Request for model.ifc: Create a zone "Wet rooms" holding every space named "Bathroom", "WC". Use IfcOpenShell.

First a look at what the model holds.

```python
import ifcopenshell

model = ifcopenshell.open("model.ifc")
print(model.schema)
seen = {}
for space in model.by_type("IfcSpace"):
    seen[space.LongName] = seen.get(space.LongName, 0) + 1
for name, count in sorted(seen.items(), key=str):
    print(count, "x", name)
print("zones:", [z.Name for z in model.by_type("IfcZone")][:20])
```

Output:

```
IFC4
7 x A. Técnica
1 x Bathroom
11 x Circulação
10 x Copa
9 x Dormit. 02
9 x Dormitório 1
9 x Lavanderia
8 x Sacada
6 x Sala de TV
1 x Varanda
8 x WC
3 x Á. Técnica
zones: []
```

```python
import ifcopenshell
import ifcopenshell.api.group
import ifcopenshell.api.root

model = ifcopenshell.open("model.ifc")

names = {"Bathroom", "WC"}
spaces = [s for s in model.by_type("IfcSpace") if s.LongName in names]

zone = ifcopenshell.api.root.create_entity(model, ifc_class="IfcZone", name="Wet rooms")
ifcopenshell.api.group.assign_group(model, products=spaces, group=zone)
print(len(spaces), "spaces in", zone.Name)

model.write("model_v2.ifc")
```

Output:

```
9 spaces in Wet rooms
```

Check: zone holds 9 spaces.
